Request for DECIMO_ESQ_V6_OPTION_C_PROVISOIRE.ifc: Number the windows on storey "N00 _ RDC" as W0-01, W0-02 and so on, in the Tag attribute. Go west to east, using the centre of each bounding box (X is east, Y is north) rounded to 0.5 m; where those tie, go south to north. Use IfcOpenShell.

First a look at what the model holds.

```python
import ifcopenshell
import ifcopenshell.util.element
import ifcopenshell.util.placement

model = ifcopenshell.open("DECIMO_ESQ_V6_OPTION_C_PROVISOIRE.ifc")
print(model.schema)
storey = next(s for s in model.by_type("IfcBuildingStorey") if s.Name == "N00 _ RDC")
windows = [e for e in ifcopenshell.util.element.get_decomposition(storey) if e.is_a("IfcWindow")]
for e in sorted(windows, key=lambda e: e.id()):
    origin = ifcopenshell.util.placement.get_local_placement(e.ObjectPlacement)[:3, 3]
    print(e.id(), e.Tag, e.Name, origin.round(2) + 0.0, sep=" | ")
```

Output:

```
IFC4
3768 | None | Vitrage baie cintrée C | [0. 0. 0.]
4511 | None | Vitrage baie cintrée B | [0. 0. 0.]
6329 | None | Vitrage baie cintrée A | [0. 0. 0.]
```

```python
import ifcopenshell
import ifcopenshell.geom
import ifcopenshell.util.element
import ifcopenshell.util.shape

model = ifcopenshell.open("DECIMO_ESQ_V6_OPTION_C_PROVISOIRE.ifc")
settings = ifcopenshell.geom.settings()
settings.set("use-world-coords", True)


def centre(element):
    shape = ifcopenshell.geom.create_shape(settings, element)
    return ifcopenshell.util.shape.get_bbox_centroid(shape.geometry)


storey = next(s for s in model.by_type("IfcBuildingStorey") if s.Name == "N00 _ RDC")
windows = [e for e in ifcopenshell.util.element.get_decomposition(storey) if e.is_a("IfcWindow")]

# Insertion points can sit at a corner or the storey origin, so sort by the geometry (in metres).
centres = {e: centre(e) for e in windows}
windows.sort(key=lambda e: (round(centres[e][0] / 0.5), centres[e][1]))

for i, e in enumerate(windows, start=1):
    number = f"W0-{i:02d}"
    e.Tag = number
    print(e.id(), number)

model.write("DECIMO_ESQ_V6_OPTION_C_PROVISOIRE_edited.ifc")
```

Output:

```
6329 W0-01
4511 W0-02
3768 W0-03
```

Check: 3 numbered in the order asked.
